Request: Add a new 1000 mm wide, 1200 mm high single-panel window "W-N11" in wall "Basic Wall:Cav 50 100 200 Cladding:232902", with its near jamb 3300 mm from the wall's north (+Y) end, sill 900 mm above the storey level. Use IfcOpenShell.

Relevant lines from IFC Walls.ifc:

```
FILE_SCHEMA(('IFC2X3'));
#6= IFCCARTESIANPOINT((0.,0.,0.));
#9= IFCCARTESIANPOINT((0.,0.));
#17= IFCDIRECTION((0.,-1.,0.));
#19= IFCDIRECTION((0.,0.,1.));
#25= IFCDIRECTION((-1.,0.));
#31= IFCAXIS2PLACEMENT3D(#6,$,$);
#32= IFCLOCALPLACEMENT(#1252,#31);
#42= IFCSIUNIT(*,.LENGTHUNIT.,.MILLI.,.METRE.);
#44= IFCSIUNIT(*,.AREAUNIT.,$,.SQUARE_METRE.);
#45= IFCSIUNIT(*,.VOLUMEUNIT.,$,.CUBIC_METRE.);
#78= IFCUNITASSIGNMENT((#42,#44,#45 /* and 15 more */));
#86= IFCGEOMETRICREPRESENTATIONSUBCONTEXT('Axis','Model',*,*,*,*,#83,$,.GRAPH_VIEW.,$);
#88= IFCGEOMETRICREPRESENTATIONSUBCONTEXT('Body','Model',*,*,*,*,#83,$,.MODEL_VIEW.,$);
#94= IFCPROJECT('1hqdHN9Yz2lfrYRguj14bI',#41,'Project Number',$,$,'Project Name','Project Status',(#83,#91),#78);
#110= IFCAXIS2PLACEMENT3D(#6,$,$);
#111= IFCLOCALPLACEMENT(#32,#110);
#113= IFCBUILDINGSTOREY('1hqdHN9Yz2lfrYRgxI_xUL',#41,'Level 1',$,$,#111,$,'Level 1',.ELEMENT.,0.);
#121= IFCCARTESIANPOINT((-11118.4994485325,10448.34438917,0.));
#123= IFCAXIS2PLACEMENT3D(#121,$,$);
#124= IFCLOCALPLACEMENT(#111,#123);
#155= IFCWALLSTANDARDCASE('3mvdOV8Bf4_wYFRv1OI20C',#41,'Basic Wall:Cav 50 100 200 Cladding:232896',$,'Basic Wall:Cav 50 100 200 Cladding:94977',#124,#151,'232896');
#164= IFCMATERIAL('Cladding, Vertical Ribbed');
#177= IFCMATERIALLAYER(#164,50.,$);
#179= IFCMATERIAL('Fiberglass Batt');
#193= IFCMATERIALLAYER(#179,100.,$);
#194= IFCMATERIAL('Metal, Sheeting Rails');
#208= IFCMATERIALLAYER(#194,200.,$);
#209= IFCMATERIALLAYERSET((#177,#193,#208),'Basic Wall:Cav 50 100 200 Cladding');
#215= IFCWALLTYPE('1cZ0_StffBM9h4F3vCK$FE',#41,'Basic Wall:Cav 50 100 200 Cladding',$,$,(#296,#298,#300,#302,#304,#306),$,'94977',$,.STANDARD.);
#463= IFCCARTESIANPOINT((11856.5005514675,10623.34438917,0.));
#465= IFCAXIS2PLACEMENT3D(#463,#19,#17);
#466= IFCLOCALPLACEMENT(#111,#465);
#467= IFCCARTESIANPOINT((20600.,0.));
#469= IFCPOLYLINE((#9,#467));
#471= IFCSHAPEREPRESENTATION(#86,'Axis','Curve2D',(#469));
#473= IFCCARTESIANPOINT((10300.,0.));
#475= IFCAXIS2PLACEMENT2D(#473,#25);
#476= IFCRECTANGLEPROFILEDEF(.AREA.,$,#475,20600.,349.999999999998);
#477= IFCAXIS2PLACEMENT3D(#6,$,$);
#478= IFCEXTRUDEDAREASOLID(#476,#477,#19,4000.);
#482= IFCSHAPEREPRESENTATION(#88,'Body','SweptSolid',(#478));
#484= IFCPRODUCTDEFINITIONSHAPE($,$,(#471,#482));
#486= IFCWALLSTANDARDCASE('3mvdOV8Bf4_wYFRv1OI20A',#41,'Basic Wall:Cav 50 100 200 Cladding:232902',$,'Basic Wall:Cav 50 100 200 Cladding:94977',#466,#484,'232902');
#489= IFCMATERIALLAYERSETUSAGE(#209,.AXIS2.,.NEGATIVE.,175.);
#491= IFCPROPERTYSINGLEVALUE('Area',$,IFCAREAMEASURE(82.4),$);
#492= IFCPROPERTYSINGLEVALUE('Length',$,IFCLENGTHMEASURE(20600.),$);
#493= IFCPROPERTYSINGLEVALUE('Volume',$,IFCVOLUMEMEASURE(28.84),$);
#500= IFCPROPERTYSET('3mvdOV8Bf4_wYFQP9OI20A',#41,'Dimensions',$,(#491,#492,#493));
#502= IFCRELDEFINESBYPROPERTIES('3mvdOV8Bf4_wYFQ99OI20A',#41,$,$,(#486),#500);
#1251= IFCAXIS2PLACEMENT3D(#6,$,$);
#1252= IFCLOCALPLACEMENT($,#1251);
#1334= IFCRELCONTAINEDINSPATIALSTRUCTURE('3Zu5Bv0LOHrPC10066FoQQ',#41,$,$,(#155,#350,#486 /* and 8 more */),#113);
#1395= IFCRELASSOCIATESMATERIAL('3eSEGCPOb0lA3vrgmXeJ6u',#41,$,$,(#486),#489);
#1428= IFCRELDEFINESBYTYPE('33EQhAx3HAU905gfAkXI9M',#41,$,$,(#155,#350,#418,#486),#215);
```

```python
import numpy as np
import ifcopenshell
import ifcopenshell.api.feature
import ifcopenshell.api.geometry
import ifcopenshell.api.pset
import ifcopenshell.api.root
import ifcopenshell.api.spatial
import ifcopenshell.api.type
import ifcopenshell.geom
import ifcopenshell.util.element
import ifcopenshell.util.placement
import ifcopenshell.util.representation
import ifcopenshell.util.shape
import ifcopenshell.util.unit

model = ifcopenshell.open("IFC Walls.ifc")
unit_scale = ifcopenshell.util.unit.calculate_unit_scale(model)
area_scale = ifcopenshell.util.unit.calculate_unit_scale(model, "AREAUNIT")
volume_scale = ifcopenshell.util.unit.calculate_unit_scale(model, "VOLUMEUNIT")
settings = ifcopenshell.geom.settings()


def volume(element):
    """Net volume in cubic metres, openings subtracted."""
    shape = ifcopenshell.geom.create_shape(settings, element)
    return ifcopenshell.util.shape.get_volume(shape.geometry)


wall = model.by_guid("3mvdOV8Bf4_wYFRv1OI20A")
storey = ifcopenshell.util.element.get_container(wall, ifc_class="IfcBuildingStorey")
context = ifcopenshell.util.representation.get_context(model, "Model", "Body", "MODEL_VIEW")
before = volume(wall)

width, height, from_end, sill = 1, 1.2, 3.3, 0.9  # metres

# The wall runs along its own X axis, and the end named is its -X end.
wall_shape = ifcopenshell.geom.create_shape(settings, wall)
x, y, z = ifcopenshell.util.shape.get_vertices(wall_shape.geometry).T
start = x.min() + from_end
face, thickness = float(y.min()), float(y.max() - y.min())
wall_matrix = ifcopenshell.util.placement.get_local_placement(wall.ObjectPlacement)
level = ifcopenshell.util.placement.get_local_placement(storey.ObjectPlacement)[2, 3]


def in_wall(x, y):
    """Placement at x, y metres in the wall's axes, at sill height."""
    matrix = wall_matrix.copy()
    matrix[:, 3] = wall_matrix @ np.array([x / unit_scale, y / unit_scale, 0.0, 1.0])
    matrix[2, 3] = level + sill / unit_scale
    return matrix


# Opening: a box that overshoots both wall faces by 50 mm.
opening = ifcopenshell.api.root.create_entity(model, ifc_class="IfcOpeningElement")
box = ifcopenshell.api.geometry.add_wall_representation(
    model, context=context, length=width, height=height, thickness=thickness + 0.1
)
ifcopenshell.api.geometry.assign_representation(model, product=opening, representation=box)
ifcopenshell.api.geometry.edit_object_placement(model, product=opening, matrix=in_wall(start, face - 0.05), is_si=False)
ifcopenshell.api.feature.add_feature(model, feature=opening, element=wall)

window = ifcopenshell.api.root.create_entity(model, ifc_class="IfcWindow", name="W-N11")
window.OverallWidth, window.OverallHeight = width / unit_scale, height / unit_scale
body = ifcopenshell.api.geometry.add_window_representation(
    model,
    context=context,
    overall_width=window.OverallWidth,
    overall_height=window.OverallHeight,
    partition_type="SINGLE_PANEL",
)
ifcopenshell.api.geometry.assign_representation(model, product=window, representation=body)
ifcopenshell.api.spatial.assign_container(model, products=[window], relating_structure=storey)
fills = ifcopenshell.api.feature.add_filling(model, opening=opening, element=window)
fills.OwnerHistory = window.OwnerHistory  # required in IFC2X3

# IFC2X3 keeps the operation on the window style.
style = ifcopenshell.api.root.create_entity(model, ifc_class="IfcWindowStyle", name="W-N11")
style.OperationType, style.ConstructionType = "SINGLE_PANEL", "NOTDEFINED"
style.ParameterTakesPrecedence = style.Sizeable = False
ifcopenshell.api.type.assign_type(model, related_objects=[window], relating_type=style)

# Centre the window in the wall's thickness.
ifcopenshell.api.geometry.edit_object_placement(model, product=window, matrix=in_wall(start, face), is_si=False)
window_shape = ifcopenshell.geom.create_shape(settings, window)
depth = ifcopenshell.util.shape.get_vertices(window_shape.geometry)[:, 1]
offset = face + thickness / 2 - (depth.min() + depth.max()) / 2
ifcopenshell.api.geometry.edit_object_placement(model, product=window, matrix=in_wall(start, offset), is_si=False)

after = volume(wall)

# Update the wall's stored quantities.
pset = model.by_id(ifcopenshell.util.element.get_pset(wall, "Dimensions", should_inherit=False)["id"])
ifcopenshell.api.pset.edit_pset(model, pset=pset, properties={
    "Area": model.create_entity("IfcAreaMeasure", after / thickness / area_scale),
    "Volume": model.create_entity("IfcVolumeMeasure", after / volume_scale),
})

print(f"wall volume {before:.3f} -> {after:.3f} m3")

model.write("IFC Walls-out.ifc")
```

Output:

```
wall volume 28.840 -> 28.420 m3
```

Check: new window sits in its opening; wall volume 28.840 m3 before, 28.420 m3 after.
